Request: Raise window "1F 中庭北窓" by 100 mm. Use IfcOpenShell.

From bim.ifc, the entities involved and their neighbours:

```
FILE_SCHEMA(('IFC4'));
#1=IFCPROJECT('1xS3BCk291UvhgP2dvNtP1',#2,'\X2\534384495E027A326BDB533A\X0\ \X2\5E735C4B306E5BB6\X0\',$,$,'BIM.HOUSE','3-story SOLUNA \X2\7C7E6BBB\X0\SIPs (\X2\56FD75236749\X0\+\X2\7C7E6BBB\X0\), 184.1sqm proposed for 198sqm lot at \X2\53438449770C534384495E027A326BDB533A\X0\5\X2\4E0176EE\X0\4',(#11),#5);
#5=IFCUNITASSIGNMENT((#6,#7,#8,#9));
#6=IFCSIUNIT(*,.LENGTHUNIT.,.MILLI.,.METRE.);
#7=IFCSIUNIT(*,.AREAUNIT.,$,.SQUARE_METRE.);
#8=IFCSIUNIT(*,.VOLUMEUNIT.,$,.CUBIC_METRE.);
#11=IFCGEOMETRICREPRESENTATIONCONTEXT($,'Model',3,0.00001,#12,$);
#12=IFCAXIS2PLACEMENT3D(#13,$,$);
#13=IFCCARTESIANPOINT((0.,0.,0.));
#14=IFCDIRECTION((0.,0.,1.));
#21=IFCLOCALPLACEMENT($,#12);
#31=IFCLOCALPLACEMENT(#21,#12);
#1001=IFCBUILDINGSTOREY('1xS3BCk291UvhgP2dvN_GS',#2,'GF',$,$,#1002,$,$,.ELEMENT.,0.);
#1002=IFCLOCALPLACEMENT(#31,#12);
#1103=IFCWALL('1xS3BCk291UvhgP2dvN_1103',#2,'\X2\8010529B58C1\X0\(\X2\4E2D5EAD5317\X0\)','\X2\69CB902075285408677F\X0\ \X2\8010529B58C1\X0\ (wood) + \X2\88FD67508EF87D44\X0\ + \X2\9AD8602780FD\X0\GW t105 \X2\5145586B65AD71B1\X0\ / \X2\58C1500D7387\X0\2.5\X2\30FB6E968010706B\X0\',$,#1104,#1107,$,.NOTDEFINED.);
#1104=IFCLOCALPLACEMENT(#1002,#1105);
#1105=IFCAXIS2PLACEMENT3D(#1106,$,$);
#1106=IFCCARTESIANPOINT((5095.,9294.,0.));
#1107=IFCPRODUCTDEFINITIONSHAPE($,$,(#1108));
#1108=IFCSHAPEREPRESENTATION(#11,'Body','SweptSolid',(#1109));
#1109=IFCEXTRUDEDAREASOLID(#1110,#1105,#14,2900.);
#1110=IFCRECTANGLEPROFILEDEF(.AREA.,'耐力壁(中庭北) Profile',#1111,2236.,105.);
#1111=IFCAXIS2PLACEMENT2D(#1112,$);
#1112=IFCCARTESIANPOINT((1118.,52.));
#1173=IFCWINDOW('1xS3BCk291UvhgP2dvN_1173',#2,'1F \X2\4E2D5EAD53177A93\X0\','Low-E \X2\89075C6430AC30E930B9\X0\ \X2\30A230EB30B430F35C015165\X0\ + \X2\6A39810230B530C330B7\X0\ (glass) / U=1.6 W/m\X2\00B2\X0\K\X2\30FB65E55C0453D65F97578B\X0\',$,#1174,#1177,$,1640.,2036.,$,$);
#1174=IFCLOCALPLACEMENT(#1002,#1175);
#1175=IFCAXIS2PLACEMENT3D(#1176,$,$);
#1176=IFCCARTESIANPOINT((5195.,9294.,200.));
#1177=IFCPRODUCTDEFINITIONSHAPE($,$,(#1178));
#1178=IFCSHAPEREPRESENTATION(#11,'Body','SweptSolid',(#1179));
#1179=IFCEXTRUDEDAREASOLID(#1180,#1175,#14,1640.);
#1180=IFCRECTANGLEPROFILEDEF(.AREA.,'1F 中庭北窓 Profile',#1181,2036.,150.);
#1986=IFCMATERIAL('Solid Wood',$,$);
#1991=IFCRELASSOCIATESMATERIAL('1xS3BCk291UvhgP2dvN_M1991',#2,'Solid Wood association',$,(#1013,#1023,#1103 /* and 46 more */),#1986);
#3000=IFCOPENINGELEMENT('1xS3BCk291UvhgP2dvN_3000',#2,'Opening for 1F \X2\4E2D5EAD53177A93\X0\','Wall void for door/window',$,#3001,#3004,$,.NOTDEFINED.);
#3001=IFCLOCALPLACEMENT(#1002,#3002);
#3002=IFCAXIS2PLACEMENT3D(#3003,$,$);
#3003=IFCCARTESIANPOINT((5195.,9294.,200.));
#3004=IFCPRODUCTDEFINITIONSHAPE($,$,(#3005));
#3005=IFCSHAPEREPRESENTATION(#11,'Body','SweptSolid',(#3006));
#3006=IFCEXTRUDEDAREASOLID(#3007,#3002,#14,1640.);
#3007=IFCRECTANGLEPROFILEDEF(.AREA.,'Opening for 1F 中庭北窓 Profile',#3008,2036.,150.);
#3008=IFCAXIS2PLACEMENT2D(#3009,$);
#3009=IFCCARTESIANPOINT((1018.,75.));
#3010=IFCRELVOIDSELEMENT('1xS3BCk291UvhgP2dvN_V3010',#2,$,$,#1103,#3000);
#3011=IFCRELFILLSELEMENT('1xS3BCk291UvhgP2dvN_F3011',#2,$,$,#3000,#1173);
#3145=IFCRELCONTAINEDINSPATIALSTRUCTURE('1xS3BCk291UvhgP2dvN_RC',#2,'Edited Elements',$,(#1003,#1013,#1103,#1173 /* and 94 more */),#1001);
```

```python
import numpy as np
import ifcopenshell
import ifcopenshell.api.geometry
import ifcopenshell.util.placement
import ifcopenshell.util.unit

model = ifcopenshell.open("bim.ifc")
unit_scale = ifcopenshell.util.unit.calculate_unit_scale(model)

window = model.by_guid("1xS3BCk291UvhgP2dvN_1173")
opening = window.FillsVoids[0].RelatingOpeningElement
dz = 0.1 / unit_scale

shift = np.array([0.0, 0.0, dz])
# The window is not placed relative to its opening, so move both.
for product in (opening, window):
    matrix = ifcopenshell.util.placement.get_local_placement(product.ObjectPlacement)
    matrix[:3, 3] += shift
    ifcopenshell.api.geometry.edit_object_placement(model, product=product, matrix=matrix, is_si=False)

print(f"moved by {dz * unit_scale:+.3f} m")

model.write("bim_v2.ifc")
```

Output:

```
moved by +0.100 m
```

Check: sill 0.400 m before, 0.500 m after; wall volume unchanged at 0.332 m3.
